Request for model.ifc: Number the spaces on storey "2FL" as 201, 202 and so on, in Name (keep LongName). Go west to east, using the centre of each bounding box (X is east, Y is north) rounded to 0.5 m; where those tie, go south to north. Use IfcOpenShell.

First a look at what the model holds.

```python
import ifcopenshell
import ifcopenshell.util.element
import ifcopenshell.util.placement

model = ifcopenshell.open("model.ifc")
print(model.schema)
storey = next(s for s in model.by_type("IfcBuildingStorey") if s.Name == "2FL")
spaces = [e for e in ifcopenshell.util.element.get_decomposition(storey) if e.is_a("IfcSpace")]
for e in sorted(spaces, key=lambda e: e.id()):
    origin = ifcopenshell.util.placement.get_local_placement(e.ObjectPlacement)[:3, 3]
    print(e.id(), e.Name, e.LongName, origin.round(2) + 0.0, sep=" | ")
```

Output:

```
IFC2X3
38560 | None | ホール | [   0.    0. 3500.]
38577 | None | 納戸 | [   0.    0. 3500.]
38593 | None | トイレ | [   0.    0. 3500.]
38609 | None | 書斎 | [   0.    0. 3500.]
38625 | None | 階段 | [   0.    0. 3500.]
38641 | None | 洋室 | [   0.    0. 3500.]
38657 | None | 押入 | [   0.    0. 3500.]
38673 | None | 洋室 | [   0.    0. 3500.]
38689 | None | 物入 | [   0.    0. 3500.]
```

```python
import ifcopenshell
import ifcopenshell.geom
import ifcopenshell.util.element
import ifcopenshell.util.shape

model = ifcopenshell.open("model.ifc")
settings = ifcopenshell.geom.settings()
settings.set("use-world-coords", True)


def centre(element):
    shape = ifcopenshell.geom.create_shape(settings, element)
    return ifcopenshell.util.shape.get_bbox_centroid(shape.geometry)


storey = next(s for s in model.by_type("IfcBuildingStorey") if s.Name == "2FL")
spaces = [e for e in ifcopenshell.util.element.get_decomposition(storey) if e.is_a("IfcSpace")]

# Insertion points can sit at a corner or the storey origin, so sort by the geometry (in metres).
centres = {e: centre(e) for e in spaces}
spaces.sort(key=lambda e: (round(centres[e][0] / 0.5), centres[e][1]))

for i, e in enumerate(spaces, start=1):
    number = f"2{i:02d}"
    e.Name = number
    print(e.id(), number)

model.write("model_edited.ifc")
```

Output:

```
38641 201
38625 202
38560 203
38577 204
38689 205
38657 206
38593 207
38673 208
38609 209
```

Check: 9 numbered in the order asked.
